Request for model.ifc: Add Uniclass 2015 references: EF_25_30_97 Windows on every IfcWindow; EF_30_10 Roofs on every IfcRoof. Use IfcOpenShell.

First a look at what the model holds.

```python
import ifcopenshell

model = ifcopenshell.open("model.ifc")
print(model.schema)
print("classifications:", [c.Name for c in model.by_type("IfcClassification")])
for ifc_class in ("IfcDoor", "IfcRoof", "IfcStair", "IfcWall", "IfcWindow"):
    print(ifc_class, len(model.by_type(ifc_class)))
```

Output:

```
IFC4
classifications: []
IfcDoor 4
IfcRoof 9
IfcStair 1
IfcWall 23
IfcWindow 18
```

```python
import ifcopenshell
import ifcopenshell.api.classification

model = ifcopenshell.open("model.ifc")

system = ifcopenshell.api.classification.add_classification(model, classification="Uniclass 2015")

codes = {
    "IfcWindow": ("EF_25_30_97", "Windows"),
    "IfcRoof": ("EF_30_10", "Roofs"),
}
for ifc_class, (code, name) in codes.items():
    products = model.by_type(ifc_class)
    ifcopenshell.api.classification.add_reference(
        model, products=products, classification=system, identification=code, name=name
    )
    print(code, len(products))

model.write("model_updated.ifc")
```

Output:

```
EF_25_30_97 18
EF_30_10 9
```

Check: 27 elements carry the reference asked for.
